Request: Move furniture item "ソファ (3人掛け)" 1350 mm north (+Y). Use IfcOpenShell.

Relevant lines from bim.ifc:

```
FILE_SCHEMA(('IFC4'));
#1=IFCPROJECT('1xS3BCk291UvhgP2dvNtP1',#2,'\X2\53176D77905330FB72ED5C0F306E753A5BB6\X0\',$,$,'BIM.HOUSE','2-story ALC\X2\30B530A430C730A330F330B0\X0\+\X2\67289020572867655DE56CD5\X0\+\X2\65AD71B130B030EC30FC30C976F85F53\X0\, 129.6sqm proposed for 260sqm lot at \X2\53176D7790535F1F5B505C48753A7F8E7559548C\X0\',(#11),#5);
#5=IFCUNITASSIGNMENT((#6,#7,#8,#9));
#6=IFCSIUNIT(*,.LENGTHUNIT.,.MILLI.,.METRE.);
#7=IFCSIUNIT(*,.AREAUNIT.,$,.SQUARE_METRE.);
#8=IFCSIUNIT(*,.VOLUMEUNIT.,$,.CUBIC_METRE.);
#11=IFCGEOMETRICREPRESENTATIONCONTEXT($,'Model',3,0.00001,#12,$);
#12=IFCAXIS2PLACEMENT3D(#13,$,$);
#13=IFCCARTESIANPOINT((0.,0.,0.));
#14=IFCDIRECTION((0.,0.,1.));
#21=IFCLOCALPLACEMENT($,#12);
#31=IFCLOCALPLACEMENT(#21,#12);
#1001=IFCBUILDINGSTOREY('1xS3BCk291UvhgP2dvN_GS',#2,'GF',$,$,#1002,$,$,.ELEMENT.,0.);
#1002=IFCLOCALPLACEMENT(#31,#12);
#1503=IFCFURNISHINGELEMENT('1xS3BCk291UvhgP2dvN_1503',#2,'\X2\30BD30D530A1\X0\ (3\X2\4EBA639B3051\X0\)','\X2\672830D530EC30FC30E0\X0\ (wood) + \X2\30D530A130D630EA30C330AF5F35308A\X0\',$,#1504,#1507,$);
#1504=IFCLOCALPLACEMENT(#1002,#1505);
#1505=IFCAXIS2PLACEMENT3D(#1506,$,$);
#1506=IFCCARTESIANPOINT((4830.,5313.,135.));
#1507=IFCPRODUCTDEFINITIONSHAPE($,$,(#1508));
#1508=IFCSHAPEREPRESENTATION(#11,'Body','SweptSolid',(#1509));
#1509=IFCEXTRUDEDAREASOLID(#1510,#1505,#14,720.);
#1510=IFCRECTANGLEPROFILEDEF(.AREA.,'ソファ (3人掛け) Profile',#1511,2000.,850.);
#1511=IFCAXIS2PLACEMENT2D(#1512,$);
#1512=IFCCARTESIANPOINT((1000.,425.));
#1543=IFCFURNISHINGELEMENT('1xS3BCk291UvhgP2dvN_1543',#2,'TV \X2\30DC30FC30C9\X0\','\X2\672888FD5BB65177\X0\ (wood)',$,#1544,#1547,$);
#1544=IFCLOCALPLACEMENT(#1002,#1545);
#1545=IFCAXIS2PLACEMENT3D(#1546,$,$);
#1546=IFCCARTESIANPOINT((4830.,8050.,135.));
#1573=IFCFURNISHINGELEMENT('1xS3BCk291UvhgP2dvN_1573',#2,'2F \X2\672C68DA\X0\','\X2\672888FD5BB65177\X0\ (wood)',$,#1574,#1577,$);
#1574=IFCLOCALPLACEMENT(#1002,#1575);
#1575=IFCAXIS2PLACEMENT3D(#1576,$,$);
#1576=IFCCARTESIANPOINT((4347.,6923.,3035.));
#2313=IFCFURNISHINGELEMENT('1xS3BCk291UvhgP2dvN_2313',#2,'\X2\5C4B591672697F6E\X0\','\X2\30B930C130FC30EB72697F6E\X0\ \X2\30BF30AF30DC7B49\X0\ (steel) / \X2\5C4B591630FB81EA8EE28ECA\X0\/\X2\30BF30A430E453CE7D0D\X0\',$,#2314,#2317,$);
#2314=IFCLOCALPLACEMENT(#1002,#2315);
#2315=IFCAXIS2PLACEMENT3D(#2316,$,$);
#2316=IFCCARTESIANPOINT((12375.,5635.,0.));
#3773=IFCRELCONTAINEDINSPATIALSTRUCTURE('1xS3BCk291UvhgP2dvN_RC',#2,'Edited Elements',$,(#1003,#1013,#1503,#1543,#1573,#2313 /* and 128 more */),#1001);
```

```python
import ifcopenshell
import ifcopenshell.api.geometry
import ifcopenshell.util.placement

model = ifcopenshell.open("bim.ifc")

item = model.by_guid("1xS3BCk291UvhgP2dvN_1503")
matrix = ifcopenshell.util.placement.get_local_placement(item.ObjectPlacement)
matrix[1, 3] += 1350.0
ifcopenshell.api.geometry.edit_object_placement(model, product=item, matrix=matrix, is_si=False)

print(ifcopenshell.util.placement.get_local_placement(item.ObjectPlacement).round(3) + 0.0)

model.write("bim_updated.ifc")
```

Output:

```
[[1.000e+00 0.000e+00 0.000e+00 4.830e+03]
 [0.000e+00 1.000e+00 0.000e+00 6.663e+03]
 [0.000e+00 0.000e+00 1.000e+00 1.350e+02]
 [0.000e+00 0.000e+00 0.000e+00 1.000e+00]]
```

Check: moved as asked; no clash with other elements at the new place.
